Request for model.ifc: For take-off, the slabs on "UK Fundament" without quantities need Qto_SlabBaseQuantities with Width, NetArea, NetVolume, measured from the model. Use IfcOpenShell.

First a look at what the model holds.

```python
import ifcopenshell
import ifcopenshell.util.element
import ifcopenshell.util.unit

model = ifcopenshell.open("model.ifc")
print(model.schema)
for unit_type in ("LENGTHUNIT", "AREAUNIT", "VOLUMEUNIT"):
    print(unit_type, ifcopenshell.util.unit.calculate_unit_scale(model, unit_type))
storey = next(s for s in model.by_type("IfcBuildingStorey") if s.Name == "UK Fundament")
slabs = [e for e in ifcopenshell.util.element.get_decomposition(storey) if e.is_a("IfcSlab")]
for e in sorted(slabs, key=lambda e: e.id()):
    print(e.id(), e.is_a(), e.Name, list(ifcopenshell.util.element.get_psets(e, qtos_only=True)), sep=" | ")
```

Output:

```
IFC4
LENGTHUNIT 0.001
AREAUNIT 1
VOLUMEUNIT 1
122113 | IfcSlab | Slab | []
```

```python
import ifcopenshell
import ifcopenshell.api.pset
import ifcopenshell.geom
import ifcopenshell.util.element
import ifcopenshell.util.shape
import ifcopenshell.util.unit

model = ifcopenshell.open("model.ifc")
unit_scale = ifcopenshell.util.unit.calculate_unit_scale(model)
area_scale = ifcopenshell.util.unit.calculate_unit_scale(model, "AREAUNIT")
volume_scale = ifcopenshell.util.unit.calculate_unit_scale(model, "VOLUMEUNIT")
settings = ifcopenshell.geom.settings()

storey = next(s for s in model.by_type("IfcBuildingStorey") if s.Name == "UK Fundament")
slabs = [e for e in ifcopenshell.util.element.get_decomposition(storey) if e.is_a("IfcSlab")]

for e in sorted(slabs, key=lambda e: e.id()):
    if ifcopenshell.util.element.get_psets(e, qtos_only=True, should_inherit=False):
        continue
    # Geometry comes back in metres, in the element's own axes.
    shape = ifcopenshell.geom.create_shape(settings, e)
    values = {
        "Width": ifcopenshell.util.shape.get_z(shape.geometry) / unit_scale,
        "NetArea": ifcopenshell.util.shape.get_footprint_area(shape.geometry) / area_scale,
        "NetVolume": ifcopenshell.util.shape.get_volume(shape.geometry) / volume_scale,
    }
    qto = ifcopenshell.api.pset.add_qto(model, product=e, name="Qto_SlabBaseQuantities")
    ifcopenshell.api.pset.edit_qto(model, qto=qto, properties=values)
    print(e.id(), {k: round(v, 3) for k, v in values.items()})

model.write("model-out.ifc")
```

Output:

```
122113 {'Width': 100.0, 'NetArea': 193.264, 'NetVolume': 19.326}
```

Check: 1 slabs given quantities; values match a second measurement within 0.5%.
